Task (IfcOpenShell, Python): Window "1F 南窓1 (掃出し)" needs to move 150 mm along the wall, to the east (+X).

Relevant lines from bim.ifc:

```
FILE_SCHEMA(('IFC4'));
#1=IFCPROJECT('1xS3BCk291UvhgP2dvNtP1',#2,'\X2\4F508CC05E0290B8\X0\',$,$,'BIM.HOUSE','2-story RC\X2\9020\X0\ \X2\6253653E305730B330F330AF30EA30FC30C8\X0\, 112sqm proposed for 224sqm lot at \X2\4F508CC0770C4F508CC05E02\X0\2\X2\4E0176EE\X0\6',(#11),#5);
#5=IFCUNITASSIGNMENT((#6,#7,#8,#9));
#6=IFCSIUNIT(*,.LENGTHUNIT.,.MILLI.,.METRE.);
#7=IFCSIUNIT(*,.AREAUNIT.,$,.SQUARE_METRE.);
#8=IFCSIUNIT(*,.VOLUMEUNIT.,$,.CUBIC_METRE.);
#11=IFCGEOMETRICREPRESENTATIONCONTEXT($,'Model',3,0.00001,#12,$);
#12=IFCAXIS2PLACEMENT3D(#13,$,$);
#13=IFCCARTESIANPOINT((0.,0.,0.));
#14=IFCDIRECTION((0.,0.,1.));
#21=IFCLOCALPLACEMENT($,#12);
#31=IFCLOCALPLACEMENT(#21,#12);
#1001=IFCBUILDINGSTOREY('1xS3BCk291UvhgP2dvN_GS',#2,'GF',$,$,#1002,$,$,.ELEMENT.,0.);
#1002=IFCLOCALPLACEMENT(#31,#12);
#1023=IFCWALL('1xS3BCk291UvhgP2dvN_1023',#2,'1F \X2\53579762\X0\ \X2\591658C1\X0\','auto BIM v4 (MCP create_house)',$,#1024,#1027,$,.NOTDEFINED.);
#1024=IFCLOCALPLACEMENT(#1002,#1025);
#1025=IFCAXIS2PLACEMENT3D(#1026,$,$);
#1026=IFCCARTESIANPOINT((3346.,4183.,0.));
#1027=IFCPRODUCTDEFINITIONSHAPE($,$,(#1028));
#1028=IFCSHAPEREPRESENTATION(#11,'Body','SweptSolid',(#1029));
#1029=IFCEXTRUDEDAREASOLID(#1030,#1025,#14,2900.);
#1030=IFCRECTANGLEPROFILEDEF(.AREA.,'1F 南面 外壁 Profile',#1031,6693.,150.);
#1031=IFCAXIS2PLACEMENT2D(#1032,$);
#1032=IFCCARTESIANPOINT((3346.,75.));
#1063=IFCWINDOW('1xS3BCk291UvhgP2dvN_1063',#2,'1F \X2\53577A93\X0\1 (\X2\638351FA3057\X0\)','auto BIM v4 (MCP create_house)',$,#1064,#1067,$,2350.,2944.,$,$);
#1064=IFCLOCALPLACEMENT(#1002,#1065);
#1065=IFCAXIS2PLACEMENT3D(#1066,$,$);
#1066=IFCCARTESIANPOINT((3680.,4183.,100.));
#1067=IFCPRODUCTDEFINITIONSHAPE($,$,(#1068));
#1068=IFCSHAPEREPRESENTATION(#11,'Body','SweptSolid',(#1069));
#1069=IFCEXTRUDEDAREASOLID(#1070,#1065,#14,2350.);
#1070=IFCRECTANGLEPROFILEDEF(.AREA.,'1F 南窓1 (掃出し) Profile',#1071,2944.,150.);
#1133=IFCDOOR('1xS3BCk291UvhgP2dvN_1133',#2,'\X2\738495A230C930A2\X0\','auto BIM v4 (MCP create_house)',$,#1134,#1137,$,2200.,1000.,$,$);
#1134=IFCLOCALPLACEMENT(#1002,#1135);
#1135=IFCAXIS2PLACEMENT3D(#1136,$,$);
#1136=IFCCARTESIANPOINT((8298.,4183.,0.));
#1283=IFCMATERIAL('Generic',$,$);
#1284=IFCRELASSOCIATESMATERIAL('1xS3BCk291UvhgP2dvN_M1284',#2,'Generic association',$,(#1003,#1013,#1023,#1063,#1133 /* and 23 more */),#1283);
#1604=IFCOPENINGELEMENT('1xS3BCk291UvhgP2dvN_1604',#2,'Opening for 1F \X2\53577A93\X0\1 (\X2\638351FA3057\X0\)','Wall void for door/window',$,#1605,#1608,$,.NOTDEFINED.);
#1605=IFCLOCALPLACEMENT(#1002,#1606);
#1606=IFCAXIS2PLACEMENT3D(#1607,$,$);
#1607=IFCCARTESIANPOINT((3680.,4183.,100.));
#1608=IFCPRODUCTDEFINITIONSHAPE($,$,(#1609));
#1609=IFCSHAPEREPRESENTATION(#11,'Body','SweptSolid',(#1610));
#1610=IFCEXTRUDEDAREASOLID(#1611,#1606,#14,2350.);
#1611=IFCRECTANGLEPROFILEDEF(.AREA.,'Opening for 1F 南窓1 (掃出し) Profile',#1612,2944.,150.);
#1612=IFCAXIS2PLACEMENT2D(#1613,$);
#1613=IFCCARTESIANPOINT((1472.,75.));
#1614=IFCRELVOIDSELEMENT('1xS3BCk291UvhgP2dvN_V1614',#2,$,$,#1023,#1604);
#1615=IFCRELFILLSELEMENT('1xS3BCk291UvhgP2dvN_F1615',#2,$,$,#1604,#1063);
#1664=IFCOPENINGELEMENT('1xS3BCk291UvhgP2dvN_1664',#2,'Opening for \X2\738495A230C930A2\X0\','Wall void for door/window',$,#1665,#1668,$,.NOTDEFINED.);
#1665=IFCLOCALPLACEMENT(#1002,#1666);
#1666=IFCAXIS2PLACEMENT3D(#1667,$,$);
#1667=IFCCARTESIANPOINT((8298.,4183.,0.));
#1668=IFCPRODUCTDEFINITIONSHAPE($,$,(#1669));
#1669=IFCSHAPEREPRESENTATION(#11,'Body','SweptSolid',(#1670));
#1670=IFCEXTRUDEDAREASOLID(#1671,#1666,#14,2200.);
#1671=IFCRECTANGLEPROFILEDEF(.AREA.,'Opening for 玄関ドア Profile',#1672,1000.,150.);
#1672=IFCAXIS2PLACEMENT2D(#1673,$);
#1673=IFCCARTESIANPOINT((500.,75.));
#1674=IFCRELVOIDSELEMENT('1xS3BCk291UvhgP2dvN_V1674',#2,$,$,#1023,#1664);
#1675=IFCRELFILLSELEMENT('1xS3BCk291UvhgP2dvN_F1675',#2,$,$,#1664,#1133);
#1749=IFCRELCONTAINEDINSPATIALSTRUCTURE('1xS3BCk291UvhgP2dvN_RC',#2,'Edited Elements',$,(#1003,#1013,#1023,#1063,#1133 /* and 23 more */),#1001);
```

```python
import ifcopenshell
import ifcopenshell.api.geometry
import ifcopenshell.util.placement
import ifcopenshell.util.unit

model = ifcopenshell.open("bim.ifc")
unit_scale = ifcopenshell.util.unit.calculate_unit_scale(model)

window = model.by_guid("1xS3BCk291UvhgP2dvN_1063")
opening = window.FillsVoids[0].RelatingOpeningElement
wall = opening.VoidsElements[0].RelatingBuildingElement

wall_matrix = ifcopenshell.util.placement.get_local_placement(wall.ObjectPlacement)
shift = wall_matrix[:3, 0] * 0.15 / unit_scale
before = ifcopenshell.util.placement.get_local_placement(window.ObjectPlacement)[:3, 3].copy()

# The window is not placed relative to its opening, so move both.
for product in (opening, window):
    matrix = ifcopenshell.util.placement.get_local_placement(product.ObjectPlacement)
    matrix[:3, 3] += shift
    ifcopenshell.api.geometry.edit_object_placement(model, product=product, matrix=matrix, is_si=False)

after = ifcopenshell.util.placement.get_local_placement(window.ObjectPlacement)[:3, 3]
print("window moved by", (after - before).round(3) + 0.0)

model.write("bim_rev.ifc")
```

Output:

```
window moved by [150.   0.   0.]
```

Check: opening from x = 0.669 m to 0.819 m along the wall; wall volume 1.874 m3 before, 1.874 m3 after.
